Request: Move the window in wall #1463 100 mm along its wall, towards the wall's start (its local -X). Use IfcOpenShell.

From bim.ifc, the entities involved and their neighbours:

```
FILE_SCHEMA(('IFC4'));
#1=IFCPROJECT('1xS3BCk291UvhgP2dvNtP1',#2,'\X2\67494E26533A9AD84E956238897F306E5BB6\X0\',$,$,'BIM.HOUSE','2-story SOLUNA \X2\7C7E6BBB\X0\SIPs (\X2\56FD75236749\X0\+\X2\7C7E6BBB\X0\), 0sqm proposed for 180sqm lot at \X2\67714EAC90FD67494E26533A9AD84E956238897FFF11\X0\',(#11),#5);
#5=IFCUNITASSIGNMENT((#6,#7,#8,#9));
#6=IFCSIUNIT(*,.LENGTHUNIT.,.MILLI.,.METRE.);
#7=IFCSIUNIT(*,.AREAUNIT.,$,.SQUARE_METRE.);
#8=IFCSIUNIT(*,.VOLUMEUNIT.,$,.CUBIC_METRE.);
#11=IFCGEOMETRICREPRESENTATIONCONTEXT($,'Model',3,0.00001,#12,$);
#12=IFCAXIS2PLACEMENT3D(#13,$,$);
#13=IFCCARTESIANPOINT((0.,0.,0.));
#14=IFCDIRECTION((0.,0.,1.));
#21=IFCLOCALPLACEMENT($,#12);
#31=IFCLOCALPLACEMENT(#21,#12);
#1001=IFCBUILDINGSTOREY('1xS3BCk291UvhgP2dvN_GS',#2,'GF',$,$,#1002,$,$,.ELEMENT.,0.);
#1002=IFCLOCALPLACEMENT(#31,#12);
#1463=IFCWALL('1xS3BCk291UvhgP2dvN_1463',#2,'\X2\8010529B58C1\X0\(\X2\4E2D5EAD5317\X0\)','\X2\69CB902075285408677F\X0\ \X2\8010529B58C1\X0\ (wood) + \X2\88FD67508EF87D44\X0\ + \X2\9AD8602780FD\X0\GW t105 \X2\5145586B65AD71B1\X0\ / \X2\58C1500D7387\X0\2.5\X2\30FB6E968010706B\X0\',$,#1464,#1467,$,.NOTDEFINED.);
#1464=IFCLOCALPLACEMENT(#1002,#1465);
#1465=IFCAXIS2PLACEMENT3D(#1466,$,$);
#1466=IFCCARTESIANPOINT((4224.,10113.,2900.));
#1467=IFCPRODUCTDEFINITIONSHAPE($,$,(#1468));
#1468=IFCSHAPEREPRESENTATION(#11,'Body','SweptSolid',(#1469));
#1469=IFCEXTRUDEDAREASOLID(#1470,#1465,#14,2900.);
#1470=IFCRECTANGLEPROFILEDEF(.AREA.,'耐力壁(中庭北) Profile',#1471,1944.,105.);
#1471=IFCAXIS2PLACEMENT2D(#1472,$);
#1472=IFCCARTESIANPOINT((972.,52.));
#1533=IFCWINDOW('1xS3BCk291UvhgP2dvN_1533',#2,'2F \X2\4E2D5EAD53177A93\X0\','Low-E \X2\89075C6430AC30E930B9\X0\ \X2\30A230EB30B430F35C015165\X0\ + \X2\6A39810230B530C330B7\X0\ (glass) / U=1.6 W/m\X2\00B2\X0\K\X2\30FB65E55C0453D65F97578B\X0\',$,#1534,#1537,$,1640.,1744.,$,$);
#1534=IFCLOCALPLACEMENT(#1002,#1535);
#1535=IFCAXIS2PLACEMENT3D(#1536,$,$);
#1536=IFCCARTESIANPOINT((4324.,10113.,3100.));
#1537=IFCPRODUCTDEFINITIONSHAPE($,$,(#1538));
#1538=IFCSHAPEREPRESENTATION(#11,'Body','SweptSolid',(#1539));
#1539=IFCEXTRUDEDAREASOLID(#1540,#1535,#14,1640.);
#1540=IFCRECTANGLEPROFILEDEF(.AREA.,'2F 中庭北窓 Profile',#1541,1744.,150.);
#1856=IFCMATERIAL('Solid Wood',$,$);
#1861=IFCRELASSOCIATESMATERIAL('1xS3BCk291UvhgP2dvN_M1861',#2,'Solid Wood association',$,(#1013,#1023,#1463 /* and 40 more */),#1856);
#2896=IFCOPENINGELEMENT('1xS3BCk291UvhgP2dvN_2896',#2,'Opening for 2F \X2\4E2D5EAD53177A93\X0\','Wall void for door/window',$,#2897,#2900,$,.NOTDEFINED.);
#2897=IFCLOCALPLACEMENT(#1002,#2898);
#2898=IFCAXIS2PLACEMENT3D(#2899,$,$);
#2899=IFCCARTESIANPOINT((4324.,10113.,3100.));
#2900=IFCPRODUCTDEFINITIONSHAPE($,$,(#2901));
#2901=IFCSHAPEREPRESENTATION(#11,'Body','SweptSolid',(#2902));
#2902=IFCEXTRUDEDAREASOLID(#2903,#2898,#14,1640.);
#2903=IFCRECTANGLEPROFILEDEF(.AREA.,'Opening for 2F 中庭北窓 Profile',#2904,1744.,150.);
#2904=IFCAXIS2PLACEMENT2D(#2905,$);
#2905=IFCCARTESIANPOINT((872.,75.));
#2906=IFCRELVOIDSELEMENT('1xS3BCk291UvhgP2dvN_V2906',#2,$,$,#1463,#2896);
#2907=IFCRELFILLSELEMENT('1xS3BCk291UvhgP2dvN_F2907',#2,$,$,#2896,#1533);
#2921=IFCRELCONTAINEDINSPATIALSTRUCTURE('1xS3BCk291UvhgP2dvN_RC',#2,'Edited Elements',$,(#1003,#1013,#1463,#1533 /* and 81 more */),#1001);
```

```python
import ifcopenshell
import ifcopenshell.api.geometry
import ifcopenshell.util.placement
import ifcopenshell.util.unit

model = ifcopenshell.open("bim.ifc")
unit_scale = ifcopenshell.util.unit.calculate_unit_scale(model)

window = model.by_guid("1xS3BCk291UvhgP2dvN_1533")
opening = window.FillsVoids[0].RelatingOpeningElement
wall = opening.VoidsElements[0].RelatingBuildingElement

wall_matrix = ifcopenshell.util.placement.get_local_placement(wall.ObjectPlacement)
shift = wall_matrix[:3, 0] * -0.1 / unit_scale
before = ifcopenshell.util.placement.get_local_placement(window.ObjectPlacement)[:3, 3].copy()

# The window is not placed relative to its opening, so move both.
for product in (opening, window):
    matrix = ifcopenshell.util.placement.get_local_placement(product.ObjectPlacement)
    matrix[:3, 3] += shift
    ifcopenshell.api.geometry.edit_object_placement(model, product=product, matrix=matrix, is_si=False)

after = ifcopenshell.util.placement.get_local_placement(window.ObjectPlacement)[:3, 3]
print("window moved by", (after - before).round(3) + 0.0)

model.write("bim_edited.ifc")
```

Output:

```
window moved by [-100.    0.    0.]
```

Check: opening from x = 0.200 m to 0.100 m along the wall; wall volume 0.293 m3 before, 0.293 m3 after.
